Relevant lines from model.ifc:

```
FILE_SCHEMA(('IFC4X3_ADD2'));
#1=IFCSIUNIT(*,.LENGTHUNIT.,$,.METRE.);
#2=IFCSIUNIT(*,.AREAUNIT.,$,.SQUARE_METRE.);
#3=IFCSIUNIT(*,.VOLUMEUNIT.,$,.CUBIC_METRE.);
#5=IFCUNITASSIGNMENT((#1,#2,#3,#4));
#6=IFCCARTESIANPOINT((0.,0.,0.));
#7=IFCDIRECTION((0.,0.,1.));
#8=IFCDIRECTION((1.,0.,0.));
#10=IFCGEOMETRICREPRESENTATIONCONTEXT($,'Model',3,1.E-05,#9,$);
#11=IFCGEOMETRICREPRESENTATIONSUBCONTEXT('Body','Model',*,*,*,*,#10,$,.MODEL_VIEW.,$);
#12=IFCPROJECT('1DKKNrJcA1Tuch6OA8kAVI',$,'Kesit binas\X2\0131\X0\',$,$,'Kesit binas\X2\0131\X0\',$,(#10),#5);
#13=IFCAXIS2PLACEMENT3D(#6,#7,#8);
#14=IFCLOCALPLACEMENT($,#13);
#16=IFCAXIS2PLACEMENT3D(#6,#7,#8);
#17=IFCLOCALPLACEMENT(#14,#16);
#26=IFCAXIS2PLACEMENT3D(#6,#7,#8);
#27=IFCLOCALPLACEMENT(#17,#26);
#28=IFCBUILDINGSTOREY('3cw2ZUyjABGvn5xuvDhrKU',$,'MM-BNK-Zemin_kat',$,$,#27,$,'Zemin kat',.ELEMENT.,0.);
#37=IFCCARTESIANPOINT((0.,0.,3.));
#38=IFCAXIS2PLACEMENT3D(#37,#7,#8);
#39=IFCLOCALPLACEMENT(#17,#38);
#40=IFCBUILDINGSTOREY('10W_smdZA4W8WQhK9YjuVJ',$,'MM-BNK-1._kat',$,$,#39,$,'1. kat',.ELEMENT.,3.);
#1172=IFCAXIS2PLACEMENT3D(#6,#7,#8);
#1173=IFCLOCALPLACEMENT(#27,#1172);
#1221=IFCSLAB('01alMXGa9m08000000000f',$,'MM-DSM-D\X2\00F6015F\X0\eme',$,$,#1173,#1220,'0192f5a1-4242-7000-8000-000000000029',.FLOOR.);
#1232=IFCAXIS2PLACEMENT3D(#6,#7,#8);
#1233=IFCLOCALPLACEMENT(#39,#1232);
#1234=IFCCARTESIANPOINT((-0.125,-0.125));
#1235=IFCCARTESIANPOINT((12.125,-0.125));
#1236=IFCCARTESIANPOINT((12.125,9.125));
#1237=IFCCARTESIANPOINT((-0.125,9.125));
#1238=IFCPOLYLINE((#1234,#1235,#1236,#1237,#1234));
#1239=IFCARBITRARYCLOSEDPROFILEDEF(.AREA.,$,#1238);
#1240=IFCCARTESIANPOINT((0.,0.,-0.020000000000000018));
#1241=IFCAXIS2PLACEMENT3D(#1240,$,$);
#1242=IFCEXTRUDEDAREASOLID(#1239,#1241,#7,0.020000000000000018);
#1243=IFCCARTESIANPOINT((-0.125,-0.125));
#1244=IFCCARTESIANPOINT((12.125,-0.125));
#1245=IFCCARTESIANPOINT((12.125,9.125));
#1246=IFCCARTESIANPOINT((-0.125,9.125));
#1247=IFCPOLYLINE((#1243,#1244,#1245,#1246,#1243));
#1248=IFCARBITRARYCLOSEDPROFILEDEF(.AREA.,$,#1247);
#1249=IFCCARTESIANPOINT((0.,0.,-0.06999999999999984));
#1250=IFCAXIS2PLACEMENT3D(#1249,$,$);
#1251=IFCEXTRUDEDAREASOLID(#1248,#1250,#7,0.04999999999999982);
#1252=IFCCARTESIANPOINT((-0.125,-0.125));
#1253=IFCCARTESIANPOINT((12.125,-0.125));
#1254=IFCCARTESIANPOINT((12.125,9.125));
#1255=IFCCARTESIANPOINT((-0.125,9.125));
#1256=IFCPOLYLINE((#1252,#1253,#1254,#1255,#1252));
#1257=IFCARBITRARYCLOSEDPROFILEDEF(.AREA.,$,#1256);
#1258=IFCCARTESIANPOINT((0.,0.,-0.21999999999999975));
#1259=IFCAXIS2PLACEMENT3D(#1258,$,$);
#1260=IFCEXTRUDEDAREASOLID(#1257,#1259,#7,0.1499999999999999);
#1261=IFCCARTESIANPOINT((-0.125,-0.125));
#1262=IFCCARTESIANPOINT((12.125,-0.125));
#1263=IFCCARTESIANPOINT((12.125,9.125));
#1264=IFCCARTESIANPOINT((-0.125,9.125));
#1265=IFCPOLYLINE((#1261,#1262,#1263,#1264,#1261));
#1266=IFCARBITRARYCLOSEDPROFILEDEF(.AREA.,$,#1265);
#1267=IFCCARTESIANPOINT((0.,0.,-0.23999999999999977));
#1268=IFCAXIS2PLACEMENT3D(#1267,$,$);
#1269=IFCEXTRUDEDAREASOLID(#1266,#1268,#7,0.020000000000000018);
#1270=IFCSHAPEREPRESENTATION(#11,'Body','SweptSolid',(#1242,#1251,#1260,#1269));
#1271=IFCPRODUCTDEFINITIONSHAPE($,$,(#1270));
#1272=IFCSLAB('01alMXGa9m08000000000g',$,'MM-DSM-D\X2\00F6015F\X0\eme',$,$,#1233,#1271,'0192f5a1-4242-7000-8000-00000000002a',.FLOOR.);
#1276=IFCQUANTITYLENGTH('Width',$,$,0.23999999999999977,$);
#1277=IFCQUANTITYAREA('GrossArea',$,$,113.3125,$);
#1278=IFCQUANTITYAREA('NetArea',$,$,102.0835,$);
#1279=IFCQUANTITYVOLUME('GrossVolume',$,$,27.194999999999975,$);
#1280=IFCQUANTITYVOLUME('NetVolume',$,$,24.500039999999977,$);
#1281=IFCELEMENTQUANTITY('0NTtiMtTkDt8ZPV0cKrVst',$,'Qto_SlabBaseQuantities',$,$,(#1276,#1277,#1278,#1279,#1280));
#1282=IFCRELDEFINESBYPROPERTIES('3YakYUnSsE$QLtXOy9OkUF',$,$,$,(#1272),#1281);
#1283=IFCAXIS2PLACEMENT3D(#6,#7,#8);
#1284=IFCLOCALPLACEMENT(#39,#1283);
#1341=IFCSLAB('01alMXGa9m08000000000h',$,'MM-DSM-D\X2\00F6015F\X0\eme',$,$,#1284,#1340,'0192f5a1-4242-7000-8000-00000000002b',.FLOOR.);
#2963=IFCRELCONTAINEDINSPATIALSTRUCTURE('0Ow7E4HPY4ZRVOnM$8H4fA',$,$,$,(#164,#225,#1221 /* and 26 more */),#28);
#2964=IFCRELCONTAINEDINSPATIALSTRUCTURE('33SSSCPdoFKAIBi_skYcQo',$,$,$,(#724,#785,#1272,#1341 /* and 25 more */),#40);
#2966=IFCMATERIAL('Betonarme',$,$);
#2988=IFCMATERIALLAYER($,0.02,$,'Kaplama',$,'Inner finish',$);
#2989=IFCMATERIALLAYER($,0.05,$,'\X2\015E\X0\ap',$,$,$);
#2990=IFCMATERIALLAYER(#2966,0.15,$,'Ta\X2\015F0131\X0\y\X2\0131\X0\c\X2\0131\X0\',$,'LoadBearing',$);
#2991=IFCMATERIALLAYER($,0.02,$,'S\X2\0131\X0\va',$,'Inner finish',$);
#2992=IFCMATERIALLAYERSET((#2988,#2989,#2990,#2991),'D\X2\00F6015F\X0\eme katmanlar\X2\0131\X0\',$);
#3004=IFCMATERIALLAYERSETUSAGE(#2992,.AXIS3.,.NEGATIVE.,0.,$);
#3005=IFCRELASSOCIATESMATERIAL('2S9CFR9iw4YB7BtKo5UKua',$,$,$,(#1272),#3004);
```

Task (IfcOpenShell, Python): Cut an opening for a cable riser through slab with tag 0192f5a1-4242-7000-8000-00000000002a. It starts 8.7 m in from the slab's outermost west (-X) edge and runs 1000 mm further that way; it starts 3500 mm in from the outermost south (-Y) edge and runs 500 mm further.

```python
import numpy as np
import ifcopenshell
import ifcopenshell.api.feature
import ifcopenshell.api.geometry
import ifcopenshell.api.pset
import ifcopenshell.api.root
import ifcopenshell.geom
import ifcopenshell.util.element
import ifcopenshell.util.placement
import ifcopenshell.util.representation
import ifcopenshell.util.shape
import ifcopenshell.util.unit

model = ifcopenshell.open("model.ifc")
unit_scale = ifcopenshell.util.unit.calculate_unit_scale(model)
area_scale = ifcopenshell.util.unit.calculate_unit_scale(model, "AREAUNIT")
volume_scale = ifcopenshell.util.unit.calculate_unit_scale(model, "VOLUMEUNIT")
settings = ifcopenshell.geom.settings()


def volume(element):
    """Net volume in cubic metres, openings subtracted."""
    shape = ifcopenshell.geom.create_shape(settings, element)
    return ifcopenshell.util.shape.get_volume(shape.geometry)


slab = model.by_id(1272)
before = volume(slab)

# Extent in the slab's own axes, in metres. The edges named are its -X and -Y sides.
slab_shape = ifcopenshell.geom.create_shape(settings, slab)
vertices = ifcopenshell.util.shape.get_vertices(slab_shape.geometry)
x_min, y_min, bottom = vertices.min(axis=0)
top = vertices[:, 2].max()

opening = ifcopenshell.api.root.create_entity(model, ifc_class="IfcOpeningElement", name="Cable riser opening", predefined_type="OPENING")
context = ifcopenshell.util.representation.get_context(model, "Model", "Body", "MODEL_VIEW")
width, depth = 1, 0.5
outline = [(0.0, 0.0), (width, 0.0), (width, depth), (0.0, depth), (0.0, 0.0)]
# Overshoot both faces by 50 mm so the cut is clean.
shape = ifcopenshell.api.geometry.add_slab_representation(
    model, context=context, depth=top - bottom + 0.1, polyline=outline
)
ifcopenshell.api.geometry.assign_representation(model, product=opening, representation=shape)

matrix = ifcopenshell.util.placement.get_local_placement(slab.ObjectPlacement)
matrix[:, 3] = matrix @ np.append(np.array([x_min + 8.7, y_min + 3.5, bottom - 0.05]) / unit_scale, 1.0)
ifcopenshell.api.geometry.edit_object_placement(model, product=opening, matrix=matrix, is_si=False)
ifcopenshell.api.feature.add_feature(model, feature=opening, element=slab)

after = volume(slab)

# Update the slab's stored quantities.
qto = model.by_id(ifcopenshell.util.element.get_pset(slab, "Qto_SlabBaseQuantities", should_inherit=False)["id"])
ifcopenshell.api.pset.edit_qto(model, qto=qto, properties={
    "NetArea": after / (top - bottom) / area_scale,
    "NetVolume": after / volume_scale,
})

print(f"slab volume {before:.3f} -> {after:.3f} m3")

model.write("model_v2.ifc")
```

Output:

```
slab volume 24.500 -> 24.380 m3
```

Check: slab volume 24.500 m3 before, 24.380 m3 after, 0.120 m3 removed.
